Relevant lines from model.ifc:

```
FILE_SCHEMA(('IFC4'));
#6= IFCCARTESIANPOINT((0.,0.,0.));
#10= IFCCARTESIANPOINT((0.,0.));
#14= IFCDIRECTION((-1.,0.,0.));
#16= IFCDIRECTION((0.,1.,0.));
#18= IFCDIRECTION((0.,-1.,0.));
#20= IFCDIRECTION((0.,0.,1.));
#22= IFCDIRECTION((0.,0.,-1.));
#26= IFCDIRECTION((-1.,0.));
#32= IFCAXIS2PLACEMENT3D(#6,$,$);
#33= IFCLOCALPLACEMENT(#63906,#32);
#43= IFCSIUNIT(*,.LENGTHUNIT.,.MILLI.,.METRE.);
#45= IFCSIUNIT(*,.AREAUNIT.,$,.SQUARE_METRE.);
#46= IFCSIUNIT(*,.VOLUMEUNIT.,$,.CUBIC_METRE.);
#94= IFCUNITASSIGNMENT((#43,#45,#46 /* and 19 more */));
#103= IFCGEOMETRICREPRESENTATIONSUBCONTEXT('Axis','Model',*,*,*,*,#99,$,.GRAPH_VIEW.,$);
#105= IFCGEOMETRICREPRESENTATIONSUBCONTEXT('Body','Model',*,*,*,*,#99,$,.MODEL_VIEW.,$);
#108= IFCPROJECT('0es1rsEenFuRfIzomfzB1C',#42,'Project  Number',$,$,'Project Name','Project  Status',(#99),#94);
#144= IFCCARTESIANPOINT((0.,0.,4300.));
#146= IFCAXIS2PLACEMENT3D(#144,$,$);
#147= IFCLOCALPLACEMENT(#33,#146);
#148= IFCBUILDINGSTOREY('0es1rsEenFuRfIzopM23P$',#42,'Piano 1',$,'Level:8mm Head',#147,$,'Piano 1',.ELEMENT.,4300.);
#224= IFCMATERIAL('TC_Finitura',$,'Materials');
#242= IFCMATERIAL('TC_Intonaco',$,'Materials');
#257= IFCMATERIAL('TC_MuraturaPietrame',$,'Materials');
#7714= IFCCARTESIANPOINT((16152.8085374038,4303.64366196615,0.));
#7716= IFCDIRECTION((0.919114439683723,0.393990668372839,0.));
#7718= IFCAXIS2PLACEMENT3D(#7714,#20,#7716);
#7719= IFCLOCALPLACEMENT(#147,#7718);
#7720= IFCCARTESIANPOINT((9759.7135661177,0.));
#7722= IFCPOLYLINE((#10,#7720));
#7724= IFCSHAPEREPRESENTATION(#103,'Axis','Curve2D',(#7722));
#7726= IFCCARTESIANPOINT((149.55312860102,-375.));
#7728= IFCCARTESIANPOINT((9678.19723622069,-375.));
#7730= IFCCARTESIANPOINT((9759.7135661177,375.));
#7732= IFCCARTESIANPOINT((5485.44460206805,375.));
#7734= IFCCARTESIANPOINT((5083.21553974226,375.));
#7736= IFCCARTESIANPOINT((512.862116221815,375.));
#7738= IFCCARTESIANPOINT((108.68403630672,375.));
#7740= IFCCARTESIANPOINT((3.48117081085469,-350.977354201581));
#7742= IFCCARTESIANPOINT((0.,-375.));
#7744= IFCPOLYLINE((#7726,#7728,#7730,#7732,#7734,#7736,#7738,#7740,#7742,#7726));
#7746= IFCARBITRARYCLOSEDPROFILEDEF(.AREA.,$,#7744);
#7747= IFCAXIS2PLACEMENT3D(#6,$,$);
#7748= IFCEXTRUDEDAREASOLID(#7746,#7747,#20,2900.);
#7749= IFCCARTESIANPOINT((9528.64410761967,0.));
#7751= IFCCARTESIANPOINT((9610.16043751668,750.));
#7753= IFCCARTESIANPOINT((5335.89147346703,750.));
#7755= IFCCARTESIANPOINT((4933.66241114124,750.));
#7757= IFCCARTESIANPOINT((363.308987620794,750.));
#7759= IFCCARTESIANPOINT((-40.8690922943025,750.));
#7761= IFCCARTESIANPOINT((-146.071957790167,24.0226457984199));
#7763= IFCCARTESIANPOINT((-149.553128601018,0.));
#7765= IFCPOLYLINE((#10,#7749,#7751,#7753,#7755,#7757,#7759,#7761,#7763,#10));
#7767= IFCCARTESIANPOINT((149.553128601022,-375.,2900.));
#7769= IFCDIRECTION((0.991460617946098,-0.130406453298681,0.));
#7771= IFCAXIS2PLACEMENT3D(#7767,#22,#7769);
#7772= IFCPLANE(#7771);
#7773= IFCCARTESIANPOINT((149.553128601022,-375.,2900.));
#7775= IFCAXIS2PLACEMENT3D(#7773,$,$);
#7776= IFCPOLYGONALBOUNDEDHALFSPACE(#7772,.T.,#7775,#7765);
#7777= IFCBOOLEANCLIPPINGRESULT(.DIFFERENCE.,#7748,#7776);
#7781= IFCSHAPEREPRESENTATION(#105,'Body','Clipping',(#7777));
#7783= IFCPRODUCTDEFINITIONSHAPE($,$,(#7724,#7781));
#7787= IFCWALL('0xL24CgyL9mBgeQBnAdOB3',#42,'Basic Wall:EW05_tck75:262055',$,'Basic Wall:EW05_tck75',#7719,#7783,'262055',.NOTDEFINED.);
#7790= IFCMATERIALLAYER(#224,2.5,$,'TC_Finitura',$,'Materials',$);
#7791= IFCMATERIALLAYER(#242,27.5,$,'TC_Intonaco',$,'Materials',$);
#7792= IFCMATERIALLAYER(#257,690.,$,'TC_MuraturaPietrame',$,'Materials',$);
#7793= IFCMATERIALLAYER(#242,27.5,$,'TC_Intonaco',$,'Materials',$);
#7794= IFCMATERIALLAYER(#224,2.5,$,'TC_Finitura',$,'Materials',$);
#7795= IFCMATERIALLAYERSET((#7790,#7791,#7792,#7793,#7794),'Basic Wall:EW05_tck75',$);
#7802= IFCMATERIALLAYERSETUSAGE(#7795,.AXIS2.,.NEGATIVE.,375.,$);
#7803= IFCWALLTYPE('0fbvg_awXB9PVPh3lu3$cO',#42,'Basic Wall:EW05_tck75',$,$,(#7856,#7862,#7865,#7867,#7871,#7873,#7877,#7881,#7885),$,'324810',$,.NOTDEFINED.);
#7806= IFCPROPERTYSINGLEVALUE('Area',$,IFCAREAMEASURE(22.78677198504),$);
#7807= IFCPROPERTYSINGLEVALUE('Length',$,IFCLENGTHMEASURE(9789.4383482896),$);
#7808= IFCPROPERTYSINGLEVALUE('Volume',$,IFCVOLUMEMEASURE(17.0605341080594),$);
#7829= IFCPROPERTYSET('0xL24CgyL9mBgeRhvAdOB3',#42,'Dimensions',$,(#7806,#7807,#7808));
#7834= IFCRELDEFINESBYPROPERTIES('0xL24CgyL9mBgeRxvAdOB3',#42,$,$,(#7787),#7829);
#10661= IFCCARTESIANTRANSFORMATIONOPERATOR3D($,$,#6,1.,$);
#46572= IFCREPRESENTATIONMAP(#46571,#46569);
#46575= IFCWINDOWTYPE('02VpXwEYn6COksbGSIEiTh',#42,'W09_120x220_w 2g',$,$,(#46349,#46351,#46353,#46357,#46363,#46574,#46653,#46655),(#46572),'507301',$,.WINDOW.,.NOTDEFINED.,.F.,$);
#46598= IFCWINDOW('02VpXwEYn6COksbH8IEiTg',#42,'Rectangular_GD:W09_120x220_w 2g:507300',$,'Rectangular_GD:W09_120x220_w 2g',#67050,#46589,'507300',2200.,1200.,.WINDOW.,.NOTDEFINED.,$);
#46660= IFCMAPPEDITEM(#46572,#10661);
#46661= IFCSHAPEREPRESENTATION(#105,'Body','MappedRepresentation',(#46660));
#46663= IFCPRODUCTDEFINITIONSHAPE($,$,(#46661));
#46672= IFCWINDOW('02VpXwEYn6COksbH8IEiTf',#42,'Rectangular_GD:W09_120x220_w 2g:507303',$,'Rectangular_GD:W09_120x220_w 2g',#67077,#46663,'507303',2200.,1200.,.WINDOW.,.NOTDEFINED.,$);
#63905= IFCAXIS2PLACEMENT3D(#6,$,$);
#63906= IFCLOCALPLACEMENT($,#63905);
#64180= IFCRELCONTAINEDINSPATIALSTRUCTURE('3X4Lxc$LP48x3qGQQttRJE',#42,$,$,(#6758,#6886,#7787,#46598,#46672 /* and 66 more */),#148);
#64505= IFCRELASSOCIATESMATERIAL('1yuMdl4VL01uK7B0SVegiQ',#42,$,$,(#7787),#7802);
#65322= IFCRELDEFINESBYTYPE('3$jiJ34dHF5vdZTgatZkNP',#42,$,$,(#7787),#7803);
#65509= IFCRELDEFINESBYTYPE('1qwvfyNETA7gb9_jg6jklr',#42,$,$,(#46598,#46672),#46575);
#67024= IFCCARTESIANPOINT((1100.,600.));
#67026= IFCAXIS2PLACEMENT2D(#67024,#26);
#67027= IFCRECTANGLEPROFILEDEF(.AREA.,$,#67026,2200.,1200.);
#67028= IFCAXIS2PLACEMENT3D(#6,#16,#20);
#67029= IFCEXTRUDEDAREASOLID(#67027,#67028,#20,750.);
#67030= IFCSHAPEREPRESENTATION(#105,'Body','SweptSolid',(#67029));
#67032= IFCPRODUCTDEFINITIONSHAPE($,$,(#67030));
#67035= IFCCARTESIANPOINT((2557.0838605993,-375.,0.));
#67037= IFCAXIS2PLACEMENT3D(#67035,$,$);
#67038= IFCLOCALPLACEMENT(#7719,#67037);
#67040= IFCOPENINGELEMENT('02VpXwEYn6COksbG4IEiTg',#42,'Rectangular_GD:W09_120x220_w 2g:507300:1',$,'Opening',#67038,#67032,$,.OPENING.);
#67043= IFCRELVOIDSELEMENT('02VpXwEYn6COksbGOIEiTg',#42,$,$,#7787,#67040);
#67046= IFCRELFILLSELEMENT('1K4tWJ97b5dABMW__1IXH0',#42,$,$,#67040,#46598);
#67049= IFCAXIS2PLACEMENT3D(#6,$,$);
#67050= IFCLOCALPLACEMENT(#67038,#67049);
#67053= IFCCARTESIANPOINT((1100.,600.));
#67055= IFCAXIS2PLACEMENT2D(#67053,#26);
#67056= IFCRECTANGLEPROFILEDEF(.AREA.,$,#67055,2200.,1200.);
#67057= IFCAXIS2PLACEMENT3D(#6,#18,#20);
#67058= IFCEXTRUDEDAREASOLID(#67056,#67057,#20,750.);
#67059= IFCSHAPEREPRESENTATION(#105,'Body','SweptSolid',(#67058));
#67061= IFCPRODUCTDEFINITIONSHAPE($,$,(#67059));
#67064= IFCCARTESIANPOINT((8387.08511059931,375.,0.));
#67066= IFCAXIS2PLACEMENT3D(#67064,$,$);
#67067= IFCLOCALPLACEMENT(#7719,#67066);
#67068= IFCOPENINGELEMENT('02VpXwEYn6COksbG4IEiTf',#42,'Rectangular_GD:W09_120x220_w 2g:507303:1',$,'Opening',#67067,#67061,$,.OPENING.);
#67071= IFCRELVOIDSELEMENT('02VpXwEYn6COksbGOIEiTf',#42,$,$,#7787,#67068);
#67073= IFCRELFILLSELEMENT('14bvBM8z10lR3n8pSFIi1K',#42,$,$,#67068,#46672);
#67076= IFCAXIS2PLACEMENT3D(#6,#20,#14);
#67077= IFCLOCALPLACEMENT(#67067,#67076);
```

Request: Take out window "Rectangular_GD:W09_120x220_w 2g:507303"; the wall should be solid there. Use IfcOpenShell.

```python
import ifcopenshell
import ifcopenshell.api.feature
import ifcopenshell.api.pset
import ifcopenshell.api.root
import ifcopenshell.geom
import ifcopenshell.util.element
import ifcopenshell.util.shape
import ifcopenshell.util.unit

model = ifcopenshell.open("model.ifc")
area_scale = ifcopenshell.util.unit.calculate_unit_scale(model, "AREAUNIT")
volume_scale = ifcopenshell.util.unit.calculate_unit_scale(model, "VOLUMEUNIT")
settings = ifcopenshell.geom.settings()


def volume(element):
    """Net volume in cubic metres, openings subtracted."""
    shape = ifcopenshell.geom.create_shape(settings, element)
    return ifcopenshell.util.shape.get_volume(shape.geometry)


window = model.by_guid("02VpXwEYn6COksbH8IEiTf")
opening = window.FillsVoids[0].RelatingOpeningElement
wall = opening.VoidsElements[0].RelatingBuildingElement
before = volume(wall)

ifcopenshell.api.root.remove_product(model, product=window)
ifcopenshell.api.feature.remove_feature(model, feature=opening)

after = volume(wall)
thickness = 0.75  # wall thickness in metres

# Update the wall's stored quantities.
pset = model.by_id(ifcopenshell.util.element.get_pset(wall, "Dimensions", should_inherit=False)["id"])
ifcopenshell.api.pset.edit_pset(model, pset=pset, properties={
    "Area": model.create_entity("IfcAreaMeasure", after / thickness / area_scale),
    "Volume": model.create_entity("IfcVolumeMeasure", after / volume_scale),
})

print(f"wall volume {before:.3f} -> {after:.3f} m3")

model.write("model_v2.ifc")
```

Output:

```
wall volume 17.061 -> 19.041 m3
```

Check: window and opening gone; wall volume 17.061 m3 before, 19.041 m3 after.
